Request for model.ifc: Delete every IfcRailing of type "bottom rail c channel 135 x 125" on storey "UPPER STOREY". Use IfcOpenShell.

First a look at what the model holds.

```python
import ifcopenshell
import ifcopenshell.util.element

model = ifcopenshell.open("model.ifc")
print(model.schema)
storey = next(s for s in model.by_type("IfcBuildingStorey") if s.Name == "UPPER STOREY")
railings = [e for e in ifcopenshell.util.element.get_decomposition(storey) if e.is_a("IfcRailing")]
seen = {}
for e in railings:
    element_type = ifcopenshell.util.element.get_type(e)
    name = element_type.Name if element_type not in (None, e) else None
    seen[name] = seen.get(name, 0) + 1
for name, count in sorted(seen.items(), key=str):
    print(count, "x", name)
```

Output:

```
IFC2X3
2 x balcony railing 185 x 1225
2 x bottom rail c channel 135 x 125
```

```python
import ifcopenshell
import ifcopenshell.api.root
import ifcopenshell.util.element

model = ifcopenshell.open("model.ifc")

storey = next(s for s in model.by_type("IfcBuildingStorey") if s.Name == "UPPER STOREY")
railings = [e for e in ifcopenshell.util.element.get_decomposition(storey) if e.is_a("IfcRailing")]
targets = [e for e in railings if (t := ifcopenshell.util.element.get_type(e)) not in (None, e) and t.Name == "bottom rail c channel 135 x 125"]

for e in targets:
    ifcopenshell.api.root.remove_product(model, product=e)
print(len(targets), "removed")

model.write("model_v2.ifc")
```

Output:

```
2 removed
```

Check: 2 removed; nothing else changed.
